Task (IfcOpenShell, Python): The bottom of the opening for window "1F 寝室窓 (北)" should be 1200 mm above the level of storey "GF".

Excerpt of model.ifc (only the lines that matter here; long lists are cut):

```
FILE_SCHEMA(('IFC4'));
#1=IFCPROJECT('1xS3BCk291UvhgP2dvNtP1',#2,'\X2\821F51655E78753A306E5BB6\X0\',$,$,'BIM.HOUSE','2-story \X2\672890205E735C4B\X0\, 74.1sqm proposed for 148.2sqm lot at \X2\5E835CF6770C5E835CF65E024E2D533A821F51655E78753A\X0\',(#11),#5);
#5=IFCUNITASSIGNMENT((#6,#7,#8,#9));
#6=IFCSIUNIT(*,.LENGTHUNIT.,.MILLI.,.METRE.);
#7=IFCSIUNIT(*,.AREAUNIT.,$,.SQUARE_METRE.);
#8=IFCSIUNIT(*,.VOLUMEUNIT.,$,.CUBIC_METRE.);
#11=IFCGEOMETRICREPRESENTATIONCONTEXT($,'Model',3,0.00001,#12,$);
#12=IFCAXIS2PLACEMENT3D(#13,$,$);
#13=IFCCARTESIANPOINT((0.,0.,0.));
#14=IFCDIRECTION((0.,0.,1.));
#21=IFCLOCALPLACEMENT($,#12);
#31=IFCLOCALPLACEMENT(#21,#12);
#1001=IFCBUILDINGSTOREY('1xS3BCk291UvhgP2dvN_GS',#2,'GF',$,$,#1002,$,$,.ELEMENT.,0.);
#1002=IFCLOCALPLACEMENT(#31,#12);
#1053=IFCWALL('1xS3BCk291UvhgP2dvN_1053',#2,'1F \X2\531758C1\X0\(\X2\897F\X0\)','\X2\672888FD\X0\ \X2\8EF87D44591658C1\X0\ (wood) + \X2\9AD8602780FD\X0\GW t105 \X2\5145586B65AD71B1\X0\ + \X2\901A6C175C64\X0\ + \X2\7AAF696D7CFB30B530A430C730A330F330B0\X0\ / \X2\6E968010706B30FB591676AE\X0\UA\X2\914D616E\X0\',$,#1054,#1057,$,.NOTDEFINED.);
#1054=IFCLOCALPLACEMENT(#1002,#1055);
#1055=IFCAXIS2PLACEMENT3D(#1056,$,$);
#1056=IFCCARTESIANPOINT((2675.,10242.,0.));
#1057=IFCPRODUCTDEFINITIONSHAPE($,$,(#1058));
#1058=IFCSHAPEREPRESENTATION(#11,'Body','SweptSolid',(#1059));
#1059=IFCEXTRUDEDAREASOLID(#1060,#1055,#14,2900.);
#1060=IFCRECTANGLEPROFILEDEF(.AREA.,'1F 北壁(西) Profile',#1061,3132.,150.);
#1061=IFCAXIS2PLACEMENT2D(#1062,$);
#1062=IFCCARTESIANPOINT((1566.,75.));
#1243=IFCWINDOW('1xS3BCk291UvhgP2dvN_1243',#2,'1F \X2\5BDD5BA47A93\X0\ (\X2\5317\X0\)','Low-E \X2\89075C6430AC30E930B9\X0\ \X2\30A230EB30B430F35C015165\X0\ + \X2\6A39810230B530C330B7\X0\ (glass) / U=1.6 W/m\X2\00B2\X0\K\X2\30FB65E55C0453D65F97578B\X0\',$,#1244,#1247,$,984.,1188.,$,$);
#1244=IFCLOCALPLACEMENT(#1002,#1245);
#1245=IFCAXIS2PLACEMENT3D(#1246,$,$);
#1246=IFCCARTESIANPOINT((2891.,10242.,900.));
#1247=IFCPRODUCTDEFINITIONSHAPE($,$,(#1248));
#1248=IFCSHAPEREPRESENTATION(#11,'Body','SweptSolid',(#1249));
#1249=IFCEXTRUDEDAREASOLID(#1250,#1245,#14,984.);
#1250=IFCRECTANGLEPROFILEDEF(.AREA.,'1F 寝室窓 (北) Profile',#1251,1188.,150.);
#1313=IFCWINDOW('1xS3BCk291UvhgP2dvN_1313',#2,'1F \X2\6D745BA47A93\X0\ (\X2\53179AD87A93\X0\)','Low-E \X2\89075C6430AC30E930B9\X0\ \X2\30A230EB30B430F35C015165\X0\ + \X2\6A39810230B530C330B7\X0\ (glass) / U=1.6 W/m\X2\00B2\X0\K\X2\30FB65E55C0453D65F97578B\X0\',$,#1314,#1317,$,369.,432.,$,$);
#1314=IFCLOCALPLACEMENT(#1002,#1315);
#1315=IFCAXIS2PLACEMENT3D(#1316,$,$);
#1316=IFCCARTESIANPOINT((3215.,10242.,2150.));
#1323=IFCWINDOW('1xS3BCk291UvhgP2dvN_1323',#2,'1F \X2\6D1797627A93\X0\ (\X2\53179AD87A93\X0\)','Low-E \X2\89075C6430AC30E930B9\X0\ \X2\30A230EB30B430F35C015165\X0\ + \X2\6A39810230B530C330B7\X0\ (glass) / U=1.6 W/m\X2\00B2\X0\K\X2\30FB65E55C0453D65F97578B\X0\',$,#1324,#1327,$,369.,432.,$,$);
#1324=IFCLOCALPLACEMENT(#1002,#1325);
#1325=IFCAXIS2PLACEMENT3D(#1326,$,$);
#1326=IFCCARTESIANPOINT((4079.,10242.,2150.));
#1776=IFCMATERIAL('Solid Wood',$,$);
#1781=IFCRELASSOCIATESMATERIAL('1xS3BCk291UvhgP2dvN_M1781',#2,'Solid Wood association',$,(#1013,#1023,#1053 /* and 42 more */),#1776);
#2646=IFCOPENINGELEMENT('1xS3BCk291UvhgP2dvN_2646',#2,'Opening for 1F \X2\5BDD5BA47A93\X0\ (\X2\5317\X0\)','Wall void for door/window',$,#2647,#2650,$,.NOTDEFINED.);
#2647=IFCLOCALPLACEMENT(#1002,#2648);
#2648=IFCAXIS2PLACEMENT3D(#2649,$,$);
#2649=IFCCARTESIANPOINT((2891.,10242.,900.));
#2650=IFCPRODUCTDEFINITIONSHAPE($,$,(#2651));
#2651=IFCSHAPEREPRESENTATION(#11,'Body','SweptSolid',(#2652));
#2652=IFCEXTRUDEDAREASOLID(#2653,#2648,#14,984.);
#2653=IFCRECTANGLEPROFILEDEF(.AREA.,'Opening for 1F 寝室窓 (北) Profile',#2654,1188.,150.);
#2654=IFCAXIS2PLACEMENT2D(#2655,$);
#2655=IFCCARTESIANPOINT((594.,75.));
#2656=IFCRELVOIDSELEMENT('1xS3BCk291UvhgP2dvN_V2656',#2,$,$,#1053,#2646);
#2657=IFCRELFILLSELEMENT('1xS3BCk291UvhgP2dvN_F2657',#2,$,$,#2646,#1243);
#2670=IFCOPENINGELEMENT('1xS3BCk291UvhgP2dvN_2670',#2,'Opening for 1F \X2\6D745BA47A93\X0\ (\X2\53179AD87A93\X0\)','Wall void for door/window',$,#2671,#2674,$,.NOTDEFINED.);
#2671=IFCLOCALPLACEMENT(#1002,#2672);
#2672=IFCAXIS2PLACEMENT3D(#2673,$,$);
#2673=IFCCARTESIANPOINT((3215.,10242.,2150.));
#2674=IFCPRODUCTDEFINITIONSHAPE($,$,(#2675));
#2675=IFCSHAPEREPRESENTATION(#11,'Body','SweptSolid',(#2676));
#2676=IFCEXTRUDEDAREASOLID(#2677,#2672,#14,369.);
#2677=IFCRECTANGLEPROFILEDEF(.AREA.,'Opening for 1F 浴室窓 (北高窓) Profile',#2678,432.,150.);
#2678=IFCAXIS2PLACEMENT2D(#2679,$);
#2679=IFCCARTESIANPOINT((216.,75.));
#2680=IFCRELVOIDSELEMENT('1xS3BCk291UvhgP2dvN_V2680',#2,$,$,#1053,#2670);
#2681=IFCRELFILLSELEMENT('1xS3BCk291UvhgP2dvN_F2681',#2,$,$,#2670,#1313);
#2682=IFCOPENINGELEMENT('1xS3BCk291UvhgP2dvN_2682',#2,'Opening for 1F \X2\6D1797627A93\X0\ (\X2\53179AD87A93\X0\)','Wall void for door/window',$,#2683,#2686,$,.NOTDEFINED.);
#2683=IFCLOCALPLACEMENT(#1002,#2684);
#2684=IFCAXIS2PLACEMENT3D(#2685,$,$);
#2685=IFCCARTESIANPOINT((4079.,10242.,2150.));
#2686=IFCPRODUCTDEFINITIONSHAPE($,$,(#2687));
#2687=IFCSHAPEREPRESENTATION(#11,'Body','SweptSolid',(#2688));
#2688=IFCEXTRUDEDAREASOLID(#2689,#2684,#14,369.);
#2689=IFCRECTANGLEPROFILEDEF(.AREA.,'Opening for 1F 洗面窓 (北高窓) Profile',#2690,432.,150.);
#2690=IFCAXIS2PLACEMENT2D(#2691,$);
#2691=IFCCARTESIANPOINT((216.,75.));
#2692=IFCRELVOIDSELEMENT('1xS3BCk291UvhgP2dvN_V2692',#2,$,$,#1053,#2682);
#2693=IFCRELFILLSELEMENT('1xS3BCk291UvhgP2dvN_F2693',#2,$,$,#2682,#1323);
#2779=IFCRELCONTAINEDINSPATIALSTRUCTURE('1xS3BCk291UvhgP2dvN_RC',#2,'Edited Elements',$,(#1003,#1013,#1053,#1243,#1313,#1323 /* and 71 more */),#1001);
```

```python
import numpy as np
import ifcopenshell
import ifcopenshell.api.geometry
import ifcopenshell.geom
import ifcopenshell.util.element
import ifcopenshell.util.placement
import ifcopenshell.util.shape
import ifcopenshell.util.unit

model = ifcopenshell.open("model.ifc")
unit_scale = ifcopenshell.util.unit.calculate_unit_scale(model)

window = model.by_guid("1xS3BCk291UvhgP2dvN_1243")
opening = window.FillsVoids[0].RelatingOpeningElement
storey = ifcopenshell.util.element.get_container(window, ifc_class="IfcBuildingStorey")
level = ifcopenshell.util.placement.get_local_placement(storey.ObjectPlacement)[2, 3]

# The opening's origin need not be at the sill, so measure its lowest point.
shape = ifcopenshell.geom.create_shape(ifcopenshell.geom.settings(), opening)
bottom = ifcopenshell.util.shape.get_shape_bottom_elevation(shape, shape.geometry) / unit_scale
dz = level + 1.2 / unit_scale - bottom

shift = np.array([0.0, 0.0, dz])
# The window is not placed relative to its opening, so move both.
for product in (opening, window):
    matrix = ifcopenshell.util.placement.get_local_placement(product.ObjectPlacement)
    matrix[:3, 3] += shift
    ifcopenshell.api.geometry.edit_object_placement(model, product=product, matrix=matrix, is_si=False)

print(f"moved by {dz * unit_scale:+.3f} m")

model.write("model_v2.ifc")
```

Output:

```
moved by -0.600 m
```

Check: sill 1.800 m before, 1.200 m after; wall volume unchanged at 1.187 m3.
